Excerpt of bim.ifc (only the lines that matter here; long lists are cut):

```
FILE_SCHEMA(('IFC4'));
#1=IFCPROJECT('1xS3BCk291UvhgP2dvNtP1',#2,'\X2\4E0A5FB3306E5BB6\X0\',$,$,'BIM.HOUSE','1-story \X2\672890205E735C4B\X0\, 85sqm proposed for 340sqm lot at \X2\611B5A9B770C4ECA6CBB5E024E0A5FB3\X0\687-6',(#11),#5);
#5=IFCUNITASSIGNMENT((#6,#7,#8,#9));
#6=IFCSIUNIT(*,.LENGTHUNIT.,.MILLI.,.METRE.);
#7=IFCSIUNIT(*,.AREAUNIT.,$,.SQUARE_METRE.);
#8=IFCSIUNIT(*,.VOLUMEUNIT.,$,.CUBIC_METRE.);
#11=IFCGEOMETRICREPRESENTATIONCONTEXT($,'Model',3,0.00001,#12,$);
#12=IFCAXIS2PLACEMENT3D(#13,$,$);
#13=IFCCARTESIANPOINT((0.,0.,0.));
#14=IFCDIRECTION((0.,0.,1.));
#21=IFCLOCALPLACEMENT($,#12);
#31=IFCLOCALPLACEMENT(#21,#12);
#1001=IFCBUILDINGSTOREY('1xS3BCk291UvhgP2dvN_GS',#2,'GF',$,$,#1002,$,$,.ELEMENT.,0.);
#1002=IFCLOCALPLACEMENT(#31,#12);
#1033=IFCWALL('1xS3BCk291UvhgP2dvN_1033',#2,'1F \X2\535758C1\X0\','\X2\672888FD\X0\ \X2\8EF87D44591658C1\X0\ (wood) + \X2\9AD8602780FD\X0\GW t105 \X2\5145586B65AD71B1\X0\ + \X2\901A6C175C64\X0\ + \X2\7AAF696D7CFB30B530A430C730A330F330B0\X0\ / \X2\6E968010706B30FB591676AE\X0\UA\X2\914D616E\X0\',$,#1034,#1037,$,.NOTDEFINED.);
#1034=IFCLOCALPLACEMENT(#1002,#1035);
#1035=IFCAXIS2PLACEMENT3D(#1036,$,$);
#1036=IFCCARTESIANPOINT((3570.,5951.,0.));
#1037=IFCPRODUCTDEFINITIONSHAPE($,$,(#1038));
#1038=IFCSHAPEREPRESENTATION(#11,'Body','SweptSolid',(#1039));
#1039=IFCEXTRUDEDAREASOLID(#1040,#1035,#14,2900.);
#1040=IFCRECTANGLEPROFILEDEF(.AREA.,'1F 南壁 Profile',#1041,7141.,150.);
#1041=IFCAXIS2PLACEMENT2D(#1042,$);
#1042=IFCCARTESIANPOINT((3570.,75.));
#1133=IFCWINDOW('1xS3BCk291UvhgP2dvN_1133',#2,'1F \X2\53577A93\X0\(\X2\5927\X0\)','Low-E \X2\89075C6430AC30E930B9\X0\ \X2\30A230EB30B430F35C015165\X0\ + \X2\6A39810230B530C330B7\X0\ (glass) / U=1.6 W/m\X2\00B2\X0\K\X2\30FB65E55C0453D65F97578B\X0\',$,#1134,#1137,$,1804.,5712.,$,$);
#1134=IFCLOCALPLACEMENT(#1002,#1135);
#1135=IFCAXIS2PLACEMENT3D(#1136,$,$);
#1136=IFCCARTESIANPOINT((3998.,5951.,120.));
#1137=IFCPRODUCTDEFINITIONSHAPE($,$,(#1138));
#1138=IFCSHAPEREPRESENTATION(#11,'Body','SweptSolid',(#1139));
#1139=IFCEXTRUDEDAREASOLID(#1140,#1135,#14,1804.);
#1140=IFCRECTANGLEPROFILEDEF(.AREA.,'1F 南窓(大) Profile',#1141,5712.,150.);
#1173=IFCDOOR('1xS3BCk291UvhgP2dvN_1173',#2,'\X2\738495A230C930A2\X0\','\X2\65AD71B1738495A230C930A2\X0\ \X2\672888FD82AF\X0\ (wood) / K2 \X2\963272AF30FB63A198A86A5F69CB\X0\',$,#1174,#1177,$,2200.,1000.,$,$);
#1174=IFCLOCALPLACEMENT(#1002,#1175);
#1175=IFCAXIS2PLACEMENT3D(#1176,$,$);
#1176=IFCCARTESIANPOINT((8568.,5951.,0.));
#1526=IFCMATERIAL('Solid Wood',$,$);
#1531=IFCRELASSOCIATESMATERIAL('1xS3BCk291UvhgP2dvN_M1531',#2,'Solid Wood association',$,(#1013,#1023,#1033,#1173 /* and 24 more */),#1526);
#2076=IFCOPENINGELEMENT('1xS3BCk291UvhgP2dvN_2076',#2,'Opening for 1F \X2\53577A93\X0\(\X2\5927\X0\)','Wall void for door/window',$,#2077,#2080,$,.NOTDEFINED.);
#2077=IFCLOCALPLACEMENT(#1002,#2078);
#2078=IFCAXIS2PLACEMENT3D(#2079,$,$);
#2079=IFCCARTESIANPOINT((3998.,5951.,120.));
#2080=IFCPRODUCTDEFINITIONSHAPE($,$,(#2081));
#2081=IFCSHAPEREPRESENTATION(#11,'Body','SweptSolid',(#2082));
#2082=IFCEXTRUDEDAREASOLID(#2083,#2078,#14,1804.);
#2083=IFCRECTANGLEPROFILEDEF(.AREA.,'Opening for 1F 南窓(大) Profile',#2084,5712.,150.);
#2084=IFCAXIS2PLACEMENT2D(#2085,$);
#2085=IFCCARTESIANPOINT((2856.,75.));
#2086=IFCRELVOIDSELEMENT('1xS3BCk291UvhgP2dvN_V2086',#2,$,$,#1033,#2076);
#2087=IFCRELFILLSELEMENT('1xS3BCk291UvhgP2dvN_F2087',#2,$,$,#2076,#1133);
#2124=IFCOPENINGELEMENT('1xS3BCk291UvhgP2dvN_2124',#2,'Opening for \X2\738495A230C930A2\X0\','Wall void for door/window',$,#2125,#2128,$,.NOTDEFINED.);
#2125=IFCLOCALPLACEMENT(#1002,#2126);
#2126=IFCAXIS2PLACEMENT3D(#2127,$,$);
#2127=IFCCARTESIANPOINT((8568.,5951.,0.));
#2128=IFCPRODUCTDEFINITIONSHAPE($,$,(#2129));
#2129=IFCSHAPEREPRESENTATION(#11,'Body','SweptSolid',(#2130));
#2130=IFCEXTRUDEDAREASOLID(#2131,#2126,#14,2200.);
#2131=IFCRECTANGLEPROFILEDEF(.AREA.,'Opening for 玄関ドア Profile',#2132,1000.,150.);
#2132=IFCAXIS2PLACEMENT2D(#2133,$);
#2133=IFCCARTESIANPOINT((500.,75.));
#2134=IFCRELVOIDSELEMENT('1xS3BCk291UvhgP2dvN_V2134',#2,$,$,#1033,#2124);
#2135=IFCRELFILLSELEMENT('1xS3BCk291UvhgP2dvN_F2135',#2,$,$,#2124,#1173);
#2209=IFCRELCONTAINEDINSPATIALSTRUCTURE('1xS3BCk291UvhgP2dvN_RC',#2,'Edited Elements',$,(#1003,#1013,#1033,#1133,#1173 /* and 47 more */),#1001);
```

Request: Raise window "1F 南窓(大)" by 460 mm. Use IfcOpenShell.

```python
import numpy as np
import ifcopenshell
import ifcopenshell.api.geometry
import ifcopenshell.util.placement
import ifcopenshell.util.unit

model = ifcopenshell.open("bim.ifc")
unit_scale = ifcopenshell.util.unit.calculate_unit_scale(model)

window = model.by_guid("1xS3BCk291UvhgP2dvN_1133")
opening = window.FillsVoids[0].RelatingOpeningElement
dz = 460.0

shift = np.array([0.0, 0.0, dz])
# The window is not placed relative to its opening, so move both.
for product in (opening, window):
    matrix = ifcopenshell.util.placement.get_local_placement(product.ObjectPlacement)
    matrix[:3, 3] += shift
    ifcopenshell.api.geometry.edit_object_placement(model, product=product, matrix=matrix, is_si=False)

print(f"moved by {dz * unit_scale:+.3f} m")

model.write("bim_updated.ifc")
```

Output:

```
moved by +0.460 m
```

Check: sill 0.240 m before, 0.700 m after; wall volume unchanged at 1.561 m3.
